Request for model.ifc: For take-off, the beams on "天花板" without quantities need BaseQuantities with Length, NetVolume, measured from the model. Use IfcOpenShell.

First a look at what the model holds.

```python
import ifcopenshell
import ifcopenshell.util.element
import ifcopenshell.util.unit

model = ifcopenshell.open("model.ifc")
print(model.schema)
for unit_type in ("LENGTHUNIT", "AREAUNIT", "VOLUMEUNIT"):
    print(unit_type, ifcopenshell.util.unit.calculate_unit_scale(model, unit_type))
storey = next(s for s in model.by_type("IfcBuildingStorey") if s.Name == "天花板")
beams = [e for e in ifcopenshell.util.element.get_decomposition(storey) if e.is_a("IfcBeam")]
for e in sorted(beams, key=lambda e: e.id()):
    print(e.id(), e.is_a(), e.Name, list(ifcopenshell.util.element.get_psets(e, qtos_only=True)), sep=" | ")
```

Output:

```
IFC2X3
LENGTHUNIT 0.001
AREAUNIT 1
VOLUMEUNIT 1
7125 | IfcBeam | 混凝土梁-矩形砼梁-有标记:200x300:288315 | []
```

```python
import ifcopenshell
import ifcopenshell.api.pset
import ifcopenshell.geom
import ifcopenshell.util.element
import ifcopenshell.util.shape
import ifcopenshell.util.unit

model = ifcopenshell.open("model.ifc")
unit_scale = ifcopenshell.util.unit.calculate_unit_scale(model)
volume_scale = ifcopenshell.util.unit.calculate_unit_scale(model, "VOLUMEUNIT")
settings = ifcopenshell.geom.settings()

storey = next(s for s in model.by_type("IfcBuildingStorey") if s.Name == "天花板")
beams = [e for e in ifcopenshell.util.element.get_decomposition(storey) if e.is_a("IfcBeam")]

for e in sorted(beams, key=lambda e: e.id()):
    if ifcopenshell.util.element.get_psets(e, qtos_only=True, should_inherit=False):
        continue
    # Geometry comes back in metres, in the element's own axes.
    shape = ifcopenshell.geom.create_shape(settings, e)
    values = {
        "Length": ifcopenshell.util.shape.get_max_xyz(shape.geometry) / unit_scale,
        "NetVolume": ifcopenshell.util.shape.get_volume(shape.geometry) / volume_scale,
    }
    qto = ifcopenshell.api.pset.add_qto(model, product=e, name="BaseQuantities")
    ifcopenshell.api.pset.edit_qto(model, qto=qto, properties=values)
    print(e.id(), {k: round(v, 3) for k, v in values.items()})

model.write("model_edited.ifc")
```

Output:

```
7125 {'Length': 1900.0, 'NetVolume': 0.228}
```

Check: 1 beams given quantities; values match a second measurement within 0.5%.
